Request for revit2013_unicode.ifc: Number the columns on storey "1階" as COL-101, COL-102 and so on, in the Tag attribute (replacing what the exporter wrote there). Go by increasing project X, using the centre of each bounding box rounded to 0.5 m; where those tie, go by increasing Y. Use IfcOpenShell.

First a look at what the model holds.

```python
import ifcopenshell
import ifcopenshell.util.element
import ifcopenshell.util.placement

model = ifcopenshell.open("revit2013_unicode.ifc")
print(model.schema)
storey = next(s for s in model.by_type("IfcBuildingStorey") if s.Name == "1階")
columns = [e for e in ifcopenshell.util.element.get_decomposition(storey) if e.is_a("IfcColumn")]
for e in sorted(columns, key=lambda e: e.id()):
    origin = ifcopenshell.util.placement.get_local_placement(e.ObjectPlacement)[:3, 3]
    print(e.id(), e.Tag, e.Name, origin.round(2) + 0.0, sep=" | ")
```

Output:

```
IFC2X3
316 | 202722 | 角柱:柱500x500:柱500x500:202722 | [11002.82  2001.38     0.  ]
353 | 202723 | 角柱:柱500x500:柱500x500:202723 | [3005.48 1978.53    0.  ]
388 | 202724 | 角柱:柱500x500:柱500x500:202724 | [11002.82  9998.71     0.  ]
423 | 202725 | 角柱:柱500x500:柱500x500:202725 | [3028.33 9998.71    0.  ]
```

```python
import ifcopenshell
import ifcopenshell.geom
import ifcopenshell.util.element
import ifcopenshell.util.shape

model = ifcopenshell.open("revit2013_unicode.ifc")
settings = ifcopenshell.geom.settings()
settings.set("use-world-coords", True)


def centre(element):
    shape = ifcopenshell.geom.create_shape(settings, element)
    return ifcopenshell.util.shape.get_bbox_centroid(shape.geometry)


storey = next(s for s in model.by_type("IfcBuildingStorey") if s.Name == "1階")
columns = [e for e in ifcopenshell.util.element.get_decomposition(storey) if e.is_a("IfcColumn")]

# Insertion points can sit at a corner or the storey origin, so sort by the geometry (in metres).
centres = {e: centre(e) for e in columns}
columns.sort(key=lambda e: (round(centres[e][0] / 0.5), centres[e][1]))

for i, e in enumerate(columns, start=1):
    number = f"COL-1{i:02d}"
    e.Tag = number
    print(e.id(), number)

model.write("revit2013_unicode_updated.ifc")
```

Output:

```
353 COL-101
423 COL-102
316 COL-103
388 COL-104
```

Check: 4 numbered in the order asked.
